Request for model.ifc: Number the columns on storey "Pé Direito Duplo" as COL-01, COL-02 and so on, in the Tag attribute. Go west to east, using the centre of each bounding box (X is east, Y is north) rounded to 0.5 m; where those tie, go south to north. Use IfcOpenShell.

First a look at what the model holds.

```python
import ifcopenshell
import ifcopenshell.util.element
import ifcopenshell.util.placement

model = ifcopenshell.open("model.ifc")
print(model.schema)
storey = next(s for s in model.by_type("IfcBuildingStorey") if s.Name == "Pé Direito Duplo")
columns = [e for e in ifcopenshell.util.element.get_decomposition(storey) if e.is_a("IfcColumn")]
for e in sorted(columns, key=lambda e: e.id()):
    origin = ifcopenshell.util.placement.get_local_placement(e.ObjectPlacement)[:3, 3]
    print(e.id(), e.Tag, e.Name, origin.round(2) + 0.0, sep=" | ")
```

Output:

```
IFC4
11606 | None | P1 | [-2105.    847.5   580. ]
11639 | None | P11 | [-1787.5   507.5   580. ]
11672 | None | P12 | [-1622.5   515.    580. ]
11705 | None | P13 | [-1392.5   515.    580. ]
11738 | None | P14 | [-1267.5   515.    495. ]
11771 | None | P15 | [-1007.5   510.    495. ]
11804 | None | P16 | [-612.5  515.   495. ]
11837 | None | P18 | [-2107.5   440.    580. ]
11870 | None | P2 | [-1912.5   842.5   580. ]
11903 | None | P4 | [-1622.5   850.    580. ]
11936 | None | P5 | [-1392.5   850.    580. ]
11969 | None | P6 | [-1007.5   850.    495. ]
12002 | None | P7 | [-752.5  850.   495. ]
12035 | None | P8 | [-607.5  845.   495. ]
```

```python
import ifcopenshell
import ifcopenshell.geom
import ifcopenshell.util.element
import ifcopenshell.util.shape

model = ifcopenshell.open("model.ifc")
settings = ifcopenshell.geom.settings()
settings.set("use-world-coords", True)


def centre(element):
    shape = ifcopenshell.geom.create_shape(settings, element)
    return ifcopenshell.util.shape.get_bbox_centroid(shape.geometry)


storey = next(s for s in model.by_type("IfcBuildingStorey") if s.Name == "Pé Direito Duplo")
columns = [e for e in ifcopenshell.util.element.get_decomposition(storey) if e.is_a("IfcColumn")]

# Insertion points can sit at a corner or the storey origin, so sort by the geometry (in metres).
centres = {e: centre(e) for e in columns}
columns.sort(key=lambda e: (round(centres[e][0] / 0.5), centres[e][1]))

for i, e in enumerate(columns, start=1):
    number = f"COL-{i:02d}"
    e.Tag = number
    print(e.id(), number)

model.write("model_v2.ifc")
```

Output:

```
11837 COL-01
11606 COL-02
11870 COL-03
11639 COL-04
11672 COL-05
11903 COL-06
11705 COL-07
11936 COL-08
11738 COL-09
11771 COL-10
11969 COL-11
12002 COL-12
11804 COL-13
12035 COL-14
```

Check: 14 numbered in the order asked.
